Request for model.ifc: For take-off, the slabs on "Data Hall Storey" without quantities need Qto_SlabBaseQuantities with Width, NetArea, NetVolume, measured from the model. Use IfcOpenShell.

First a look at what the model holds.

```python
import ifcopenshell
import ifcopenshell.util.element
import ifcopenshell.util.unit

model = ifcopenshell.open("model.ifc")
print(model.schema)
for unit_type in ("LENGTHUNIT", "AREAUNIT", "VOLUMEUNIT"):
    print(unit_type, ifcopenshell.util.unit.calculate_unit_scale(model, unit_type))
storey = next(s for s in model.by_type("IfcBuildingStorey") if s.Name == "Data Hall Storey")
slabs = [e for e in ifcopenshell.util.element.get_decomposition(storey) if e.is_a("IfcSlab")]
for e in sorted(slabs, key=lambda e: e.id()):
    print(e.id(), e.is_a(), e.Name, list(ifcopenshell.util.element.get_psets(e, qtos_only=True)), sep=" | ")
```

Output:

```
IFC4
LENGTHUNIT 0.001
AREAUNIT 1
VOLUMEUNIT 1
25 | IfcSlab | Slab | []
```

```python
import ifcopenshell
import ifcopenshell.api.pset
import ifcopenshell.geom
import ifcopenshell.util.element
import ifcopenshell.util.shape
import ifcopenshell.util.unit

model = ifcopenshell.open("model.ifc")
unit_scale = ifcopenshell.util.unit.calculate_unit_scale(model)
area_scale = ifcopenshell.util.unit.calculate_unit_scale(model, "AREAUNIT")
volume_scale = ifcopenshell.util.unit.calculate_unit_scale(model, "VOLUMEUNIT")
settings = ifcopenshell.geom.settings()

storey = next(s for s in model.by_type("IfcBuildingStorey") if s.Name == "Data Hall Storey")
slabs = [e for e in ifcopenshell.util.element.get_decomposition(storey) if e.is_a("IfcSlab")]

for e in sorted(slabs, key=lambda e: e.id()):
    if ifcopenshell.util.element.get_psets(e, qtos_only=True, should_inherit=False):
        continue
    # Geometry comes back in metres, in the element's own axes.
    shape = ifcopenshell.geom.create_shape(settings, e)
    values = {
        "Width": ifcopenshell.util.shape.get_z(shape.geometry) / unit_scale,
        "NetArea": ifcopenshell.util.shape.get_footprint_area(shape.geometry) / area_scale,
        "NetVolume": ifcopenshell.util.shape.get_volume(shape.geometry) / volume_scale,
    }
    qto = ifcopenshell.api.pset.add_qto(model, product=e, name="Qto_SlabBaseQuantities")
    ifcopenshell.api.pset.edit_qto(model, qto=qto, properties=values)
    print(e.id(), {k: round(v, 3) for k, v in values.items()})

model.write("model_rev.ifc")
```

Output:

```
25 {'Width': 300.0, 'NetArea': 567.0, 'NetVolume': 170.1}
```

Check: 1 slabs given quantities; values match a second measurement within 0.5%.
